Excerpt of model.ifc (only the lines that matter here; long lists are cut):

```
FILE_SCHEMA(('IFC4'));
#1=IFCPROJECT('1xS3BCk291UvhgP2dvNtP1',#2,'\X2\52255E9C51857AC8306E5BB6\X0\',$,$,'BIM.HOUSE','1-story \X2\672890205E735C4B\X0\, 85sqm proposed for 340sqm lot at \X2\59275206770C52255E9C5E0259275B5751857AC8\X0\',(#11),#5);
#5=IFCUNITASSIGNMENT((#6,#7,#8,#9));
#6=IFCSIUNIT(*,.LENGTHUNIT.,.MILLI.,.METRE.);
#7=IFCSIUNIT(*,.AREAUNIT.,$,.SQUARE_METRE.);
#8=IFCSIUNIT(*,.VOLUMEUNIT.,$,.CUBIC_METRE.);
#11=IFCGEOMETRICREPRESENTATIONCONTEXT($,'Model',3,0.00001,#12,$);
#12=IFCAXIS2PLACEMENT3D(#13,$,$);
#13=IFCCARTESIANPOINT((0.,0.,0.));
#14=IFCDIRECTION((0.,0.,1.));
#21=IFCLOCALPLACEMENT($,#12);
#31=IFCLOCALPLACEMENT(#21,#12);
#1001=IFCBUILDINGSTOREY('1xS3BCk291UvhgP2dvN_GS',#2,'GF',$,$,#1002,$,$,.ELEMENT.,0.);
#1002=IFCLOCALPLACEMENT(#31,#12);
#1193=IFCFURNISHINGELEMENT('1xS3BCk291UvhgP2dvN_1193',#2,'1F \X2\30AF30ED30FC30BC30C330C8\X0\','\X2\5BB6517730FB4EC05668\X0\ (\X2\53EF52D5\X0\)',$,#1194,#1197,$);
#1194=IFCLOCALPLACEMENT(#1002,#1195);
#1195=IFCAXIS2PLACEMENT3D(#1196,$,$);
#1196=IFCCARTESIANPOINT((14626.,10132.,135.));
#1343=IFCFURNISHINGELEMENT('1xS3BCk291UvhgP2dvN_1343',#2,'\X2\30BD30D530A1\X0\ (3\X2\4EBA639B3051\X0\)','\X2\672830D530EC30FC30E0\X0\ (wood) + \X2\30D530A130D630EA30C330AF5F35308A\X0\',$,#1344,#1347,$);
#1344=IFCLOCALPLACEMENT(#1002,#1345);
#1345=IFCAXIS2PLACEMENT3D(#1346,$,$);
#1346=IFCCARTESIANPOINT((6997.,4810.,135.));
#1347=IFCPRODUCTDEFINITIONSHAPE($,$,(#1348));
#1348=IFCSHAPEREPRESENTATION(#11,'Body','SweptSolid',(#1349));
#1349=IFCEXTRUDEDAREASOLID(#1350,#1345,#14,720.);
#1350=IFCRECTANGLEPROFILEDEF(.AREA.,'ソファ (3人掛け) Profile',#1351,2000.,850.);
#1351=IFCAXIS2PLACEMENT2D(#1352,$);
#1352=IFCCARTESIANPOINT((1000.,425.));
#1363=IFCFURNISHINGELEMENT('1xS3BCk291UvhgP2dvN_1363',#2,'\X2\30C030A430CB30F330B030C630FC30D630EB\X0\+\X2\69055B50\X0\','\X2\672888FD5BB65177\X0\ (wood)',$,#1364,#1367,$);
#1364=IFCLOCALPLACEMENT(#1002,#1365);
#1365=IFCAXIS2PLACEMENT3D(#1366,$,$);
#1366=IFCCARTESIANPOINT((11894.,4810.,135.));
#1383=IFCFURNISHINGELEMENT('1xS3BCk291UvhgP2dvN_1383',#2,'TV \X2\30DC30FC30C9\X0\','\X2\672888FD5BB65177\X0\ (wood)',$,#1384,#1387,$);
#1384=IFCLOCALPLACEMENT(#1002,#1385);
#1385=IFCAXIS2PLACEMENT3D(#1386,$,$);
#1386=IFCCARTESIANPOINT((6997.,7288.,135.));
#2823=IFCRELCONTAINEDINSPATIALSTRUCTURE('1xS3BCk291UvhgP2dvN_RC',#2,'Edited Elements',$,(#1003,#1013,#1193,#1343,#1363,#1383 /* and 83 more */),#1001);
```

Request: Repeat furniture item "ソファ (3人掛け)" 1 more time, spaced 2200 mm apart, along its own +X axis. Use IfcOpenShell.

```python
import ifcopenshell
import ifcopenshell.api.geometry
import ifcopenshell.api.root
import ifcopenshell.util.element
import ifcopenshell.util.placement
import ifcopenshell.util.unit

model = ifcopenshell.open("model.ifc")
unit_scale = ifcopenshell.util.unit.calculate_unit_scale(model)


def reuse_history(source, copy):
    """copy_class also copies each property set's owner history, people and application; keep the originals."""
    for rel in copy.IsDefinedBy:
        if rel.is_a("IfcRelDefinesByProperties") and (history := rel.RelatingPropertyDefinition.OwnerHistory):
            rel.RelatingPropertyDefinition.OwnerHistory = source.OwnerHistory
            ifcopenshell.util.element.remove_deep2(model, history)


source = model.by_guid("1xS3BCk291UvhgP2dvN_1343")
base = ifcopenshell.util.placement.get_local_placement(source.ObjectPlacement)
step = base[:3, 0] * 2.2 / unit_scale

for i in range(1, 2):
    copy = ifcopenshell.api.root.copy_class(model, product=source)
    copy.Representation = ifcopenshell.util.element.copy_deep(
        model, source.Representation, exclude=["IfcGeometricRepresentationContext", "IfcRepresentationMap"]
    )
    reuse_history(source, copy)
    matrix = base.copy()
    matrix[:3, 3] += i * step
    print("added at", matrix[:3, 3].round(3) + 0.0)
    ifcopenshell.api.geometry.edit_object_placement(model, product=copy, matrix=matrix, is_si=False)

model.write("model-out.ifc")
```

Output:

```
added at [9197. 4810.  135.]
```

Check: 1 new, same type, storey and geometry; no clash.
